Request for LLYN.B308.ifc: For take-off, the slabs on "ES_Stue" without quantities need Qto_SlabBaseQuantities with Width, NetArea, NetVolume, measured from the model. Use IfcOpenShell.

First a look at what the model holds.

```python
import ifcopenshell
import ifcopenshell.util.element
import ifcopenshell.util.unit

model = ifcopenshell.open("LLYN.B308.ifc")
print(model.schema)
for unit_type in ("LENGTHUNIT", "AREAUNIT", "VOLUMEUNIT"):
    print(unit_type, ifcopenshell.util.unit.calculate_unit_scale(model, unit_type))
storey = next(s for s in model.by_type("IfcBuildingStorey") if s.Name == "ES_Stue")
slabs = [e for e in ifcopenshell.util.element.get_decomposition(storey) if e.is_a("IfcSlab")]
for e in sorted(slabs, key=lambda e: e.id()):
    print(e.id(), e.is_a(), e.Name, list(ifcopenshell.util.element.get_psets(e, qtos_only=True)), sep=" | ")
```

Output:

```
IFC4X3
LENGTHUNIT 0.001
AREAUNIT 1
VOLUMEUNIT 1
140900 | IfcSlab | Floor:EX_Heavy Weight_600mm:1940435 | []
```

```python
import ifcopenshell
import ifcopenshell.api.pset
import ifcopenshell.geom
import ifcopenshell.util.element
import ifcopenshell.util.shape
import ifcopenshell.util.unit

model = ifcopenshell.open("LLYN.B308.ifc")
unit_scale = ifcopenshell.util.unit.calculate_unit_scale(model)
area_scale = ifcopenshell.util.unit.calculate_unit_scale(model, "AREAUNIT")
volume_scale = ifcopenshell.util.unit.calculate_unit_scale(model, "VOLUMEUNIT")
settings = ifcopenshell.geom.settings()

storey = next(s for s in model.by_type("IfcBuildingStorey") if s.Name == "ES_Stue")
slabs = [e for e in ifcopenshell.util.element.get_decomposition(storey) if e.is_a("IfcSlab")]

for e in sorted(slabs, key=lambda e: e.id()):
    if ifcopenshell.util.element.get_psets(e, qtos_only=True, should_inherit=False):
        continue
    # Geometry comes back in metres, in the element's own axes.
    shape = ifcopenshell.geom.create_shape(settings, e)
    values = {
        "Width": ifcopenshell.util.shape.get_z(shape.geometry) / unit_scale,
        "NetArea": ifcopenshell.util.shape.get_footprint_area(shape.geometry) / area_scale,
        "NetVolume": ifcopenshell.util.shape.get_volume(shape.geometry) / volume_scale,
    }
    qto = ifcopenshell.api.pset.add_qto(model, product=e, name="Qto_SlabBaseQuantities")
    ifcopenshell.api.pset.edit_qto(model, qto=qto, properties=values)
    print(e.id(), {k: round(v, 3) for k, v in values.items()})

model.write("LLYN.B308-out.ifc")
```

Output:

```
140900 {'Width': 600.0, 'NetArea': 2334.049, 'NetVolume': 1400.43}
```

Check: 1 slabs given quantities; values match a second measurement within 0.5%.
